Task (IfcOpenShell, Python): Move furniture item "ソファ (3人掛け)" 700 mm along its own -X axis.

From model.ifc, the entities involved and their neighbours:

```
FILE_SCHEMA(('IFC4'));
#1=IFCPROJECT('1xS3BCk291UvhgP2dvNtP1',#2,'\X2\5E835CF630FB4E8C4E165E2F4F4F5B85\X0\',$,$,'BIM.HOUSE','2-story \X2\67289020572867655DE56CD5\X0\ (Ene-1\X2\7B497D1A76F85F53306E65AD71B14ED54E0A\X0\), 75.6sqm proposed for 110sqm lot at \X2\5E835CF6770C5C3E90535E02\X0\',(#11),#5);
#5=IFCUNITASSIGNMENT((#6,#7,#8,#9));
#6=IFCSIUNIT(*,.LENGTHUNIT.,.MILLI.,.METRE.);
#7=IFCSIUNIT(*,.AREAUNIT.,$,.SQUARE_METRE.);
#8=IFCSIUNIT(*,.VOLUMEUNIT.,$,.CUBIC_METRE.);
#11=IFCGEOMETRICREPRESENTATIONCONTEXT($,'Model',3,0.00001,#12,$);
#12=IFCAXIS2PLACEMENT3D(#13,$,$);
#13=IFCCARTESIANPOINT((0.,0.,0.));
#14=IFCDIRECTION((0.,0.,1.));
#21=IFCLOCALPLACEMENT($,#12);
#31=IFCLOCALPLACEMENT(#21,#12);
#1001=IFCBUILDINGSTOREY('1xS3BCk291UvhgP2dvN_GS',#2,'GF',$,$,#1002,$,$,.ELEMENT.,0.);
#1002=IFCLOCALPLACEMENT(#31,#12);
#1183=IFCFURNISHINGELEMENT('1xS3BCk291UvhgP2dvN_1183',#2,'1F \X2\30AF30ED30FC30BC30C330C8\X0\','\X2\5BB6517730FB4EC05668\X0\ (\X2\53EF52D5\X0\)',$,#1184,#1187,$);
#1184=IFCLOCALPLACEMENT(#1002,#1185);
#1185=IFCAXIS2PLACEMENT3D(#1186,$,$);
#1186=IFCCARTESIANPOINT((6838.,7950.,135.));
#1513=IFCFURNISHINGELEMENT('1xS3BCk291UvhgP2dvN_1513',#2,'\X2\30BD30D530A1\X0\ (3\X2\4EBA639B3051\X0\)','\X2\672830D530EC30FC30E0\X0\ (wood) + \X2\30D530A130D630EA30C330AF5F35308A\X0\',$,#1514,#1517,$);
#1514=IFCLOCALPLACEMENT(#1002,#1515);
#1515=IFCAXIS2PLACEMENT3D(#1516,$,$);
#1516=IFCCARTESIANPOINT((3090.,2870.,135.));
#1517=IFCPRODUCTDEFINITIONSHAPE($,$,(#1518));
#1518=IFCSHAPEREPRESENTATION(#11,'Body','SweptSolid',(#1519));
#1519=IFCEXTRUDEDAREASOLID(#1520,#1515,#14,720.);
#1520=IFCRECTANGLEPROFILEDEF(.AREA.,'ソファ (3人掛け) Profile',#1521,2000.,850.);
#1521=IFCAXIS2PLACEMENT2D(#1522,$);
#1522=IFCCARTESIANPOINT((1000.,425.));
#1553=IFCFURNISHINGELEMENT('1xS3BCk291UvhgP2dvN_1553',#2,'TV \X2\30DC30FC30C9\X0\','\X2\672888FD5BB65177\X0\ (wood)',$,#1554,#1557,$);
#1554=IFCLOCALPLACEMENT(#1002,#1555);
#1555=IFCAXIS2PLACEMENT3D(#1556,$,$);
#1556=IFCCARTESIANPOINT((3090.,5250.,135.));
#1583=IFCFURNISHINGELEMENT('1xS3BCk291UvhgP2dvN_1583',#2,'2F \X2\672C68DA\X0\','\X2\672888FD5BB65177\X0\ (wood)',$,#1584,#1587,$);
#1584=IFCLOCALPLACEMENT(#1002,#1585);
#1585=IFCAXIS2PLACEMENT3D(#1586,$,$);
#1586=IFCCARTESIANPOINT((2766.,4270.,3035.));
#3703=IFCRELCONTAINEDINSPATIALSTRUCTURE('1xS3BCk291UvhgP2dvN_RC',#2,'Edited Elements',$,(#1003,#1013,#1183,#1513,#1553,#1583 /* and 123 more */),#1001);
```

```python
import ifcopenshell
import ifcopenshell.api.geometry
import ifcopenshell.util.placement
import ifcopenshell.util.unit

model = ifcopenshell.open("model.ifc")
unit_scale = ifcopenshell.util.unit.calculate_unit_scale(model)

item = model.by_id(1513)
matrix = ifcopenshell.util.placement.get_local_placement(item.ObjectPlacement)
matrix[:3, 3] -= matrix[:3, 0] * 0.7 / unit_scale
ifcopenshell.api.geometry.edit_object_placement(model, product=item, matrix=matrix, is_si=False)

print(ifcopenshell.util.placement.get_local_placement(item.ObjectPlacement).round(3) + 0.0)

model.write("model_edited.ifc")
```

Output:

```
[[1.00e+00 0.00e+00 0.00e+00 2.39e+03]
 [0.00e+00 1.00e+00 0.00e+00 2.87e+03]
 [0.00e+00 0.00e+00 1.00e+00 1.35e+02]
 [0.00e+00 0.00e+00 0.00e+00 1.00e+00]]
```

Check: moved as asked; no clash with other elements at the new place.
